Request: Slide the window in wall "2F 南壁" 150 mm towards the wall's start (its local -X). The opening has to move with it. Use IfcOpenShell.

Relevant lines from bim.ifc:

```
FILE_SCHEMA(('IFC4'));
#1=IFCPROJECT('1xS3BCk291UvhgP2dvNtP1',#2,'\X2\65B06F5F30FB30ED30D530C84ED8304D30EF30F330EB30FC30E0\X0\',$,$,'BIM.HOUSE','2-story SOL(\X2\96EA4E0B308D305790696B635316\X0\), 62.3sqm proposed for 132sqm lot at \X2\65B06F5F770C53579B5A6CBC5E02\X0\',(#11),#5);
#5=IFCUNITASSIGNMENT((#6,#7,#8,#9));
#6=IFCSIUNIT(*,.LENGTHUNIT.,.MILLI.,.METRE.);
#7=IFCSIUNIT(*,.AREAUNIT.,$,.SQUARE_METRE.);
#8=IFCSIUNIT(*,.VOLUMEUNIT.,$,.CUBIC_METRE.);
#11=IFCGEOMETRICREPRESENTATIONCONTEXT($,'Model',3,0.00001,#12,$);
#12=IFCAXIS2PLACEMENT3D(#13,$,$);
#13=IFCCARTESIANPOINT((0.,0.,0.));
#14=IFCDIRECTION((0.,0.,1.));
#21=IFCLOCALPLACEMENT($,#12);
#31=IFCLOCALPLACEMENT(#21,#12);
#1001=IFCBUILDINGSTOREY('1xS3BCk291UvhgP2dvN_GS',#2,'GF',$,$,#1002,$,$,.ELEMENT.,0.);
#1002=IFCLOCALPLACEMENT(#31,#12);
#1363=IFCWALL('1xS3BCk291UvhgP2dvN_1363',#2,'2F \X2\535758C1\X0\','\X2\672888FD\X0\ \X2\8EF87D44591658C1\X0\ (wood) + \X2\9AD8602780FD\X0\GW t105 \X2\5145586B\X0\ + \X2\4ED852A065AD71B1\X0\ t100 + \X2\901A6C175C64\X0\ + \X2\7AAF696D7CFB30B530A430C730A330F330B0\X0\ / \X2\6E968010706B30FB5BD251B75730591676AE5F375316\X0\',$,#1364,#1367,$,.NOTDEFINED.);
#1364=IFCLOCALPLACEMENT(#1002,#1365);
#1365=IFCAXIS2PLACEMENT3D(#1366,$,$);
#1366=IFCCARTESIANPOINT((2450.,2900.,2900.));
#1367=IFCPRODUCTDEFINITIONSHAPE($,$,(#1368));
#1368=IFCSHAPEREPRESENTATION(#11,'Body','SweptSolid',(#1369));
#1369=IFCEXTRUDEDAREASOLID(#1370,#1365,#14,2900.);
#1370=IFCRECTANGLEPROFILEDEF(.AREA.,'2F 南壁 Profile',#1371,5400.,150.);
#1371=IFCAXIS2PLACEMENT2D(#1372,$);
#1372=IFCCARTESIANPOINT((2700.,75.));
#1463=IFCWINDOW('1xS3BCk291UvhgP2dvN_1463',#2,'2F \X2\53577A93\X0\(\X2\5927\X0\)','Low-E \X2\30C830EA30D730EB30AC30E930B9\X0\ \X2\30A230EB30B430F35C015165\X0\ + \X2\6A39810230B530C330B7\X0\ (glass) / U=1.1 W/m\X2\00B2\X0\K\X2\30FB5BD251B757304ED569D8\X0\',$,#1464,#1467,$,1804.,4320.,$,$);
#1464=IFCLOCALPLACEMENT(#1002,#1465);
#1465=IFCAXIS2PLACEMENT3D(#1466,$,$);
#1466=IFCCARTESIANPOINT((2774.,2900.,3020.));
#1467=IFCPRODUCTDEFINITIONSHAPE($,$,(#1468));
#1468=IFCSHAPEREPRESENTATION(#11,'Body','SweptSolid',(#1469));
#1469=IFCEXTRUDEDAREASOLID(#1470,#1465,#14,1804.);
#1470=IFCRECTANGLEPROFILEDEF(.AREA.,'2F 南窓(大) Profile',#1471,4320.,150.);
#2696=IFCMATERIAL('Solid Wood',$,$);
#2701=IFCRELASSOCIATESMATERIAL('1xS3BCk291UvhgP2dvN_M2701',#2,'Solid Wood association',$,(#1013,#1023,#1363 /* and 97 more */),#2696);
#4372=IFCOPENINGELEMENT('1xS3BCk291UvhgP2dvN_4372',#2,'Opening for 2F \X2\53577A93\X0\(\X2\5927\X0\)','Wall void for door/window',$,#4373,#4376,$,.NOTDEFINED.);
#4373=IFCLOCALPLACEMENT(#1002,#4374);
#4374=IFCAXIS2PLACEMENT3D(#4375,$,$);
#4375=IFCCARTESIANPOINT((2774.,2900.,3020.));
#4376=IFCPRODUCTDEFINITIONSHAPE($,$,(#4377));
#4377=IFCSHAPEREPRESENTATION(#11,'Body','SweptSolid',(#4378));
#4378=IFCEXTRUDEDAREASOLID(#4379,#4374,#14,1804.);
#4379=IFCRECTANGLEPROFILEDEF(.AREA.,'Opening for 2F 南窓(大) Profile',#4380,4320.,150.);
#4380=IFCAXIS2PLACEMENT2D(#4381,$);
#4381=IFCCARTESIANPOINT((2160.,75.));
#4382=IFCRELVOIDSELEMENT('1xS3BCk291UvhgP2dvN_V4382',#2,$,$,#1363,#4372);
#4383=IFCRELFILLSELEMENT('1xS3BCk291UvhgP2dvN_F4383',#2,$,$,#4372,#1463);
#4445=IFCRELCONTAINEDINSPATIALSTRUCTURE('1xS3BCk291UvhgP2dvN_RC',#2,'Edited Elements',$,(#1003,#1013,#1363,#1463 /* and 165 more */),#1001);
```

```python
import ifcopenshell
import ifcopenshell.api.geometry
import ifcopenshell.util.placement

model = ifcopenshell.open("bim.ifc")

window = model.by_guid("1xS3BCk291UvhgP2dvN_1463")
opening = window.FillsVoids[0].RelatingOpeningElement
wall = opening.VoidsElements[0].RelatingBuildingElement

wall_matrix = ifcopenshell.util.placement.get_local_placement(wall.ObjectPlacement)
shift = wall_matrix[:3, 0] * -150.0
before = ifcopenshell.util.placement.get_local_placement(window.ObjectPlacement)[:3, 3].copy()

# The window is not placed relative to its opening, so move both.
for product in (opening, window):
    matrix = ifcopenshell.util.placement.get_local_placement(product.ObjectPlacement)
    matrix[:3, 3] += shift
    ifcopenshell.api.geometry.edit_object_placement(model, product=product, matrix=matrix, is_si=False)

after = ifcopenshell.util.placement.get_local_placement(window.ObjectPlacement)[:3, 3]
print("window moved by", (after - before).round(3) + 0.0)

model.write("bim_rev.ifc")
```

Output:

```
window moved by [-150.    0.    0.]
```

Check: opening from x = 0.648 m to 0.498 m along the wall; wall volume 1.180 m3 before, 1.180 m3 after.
